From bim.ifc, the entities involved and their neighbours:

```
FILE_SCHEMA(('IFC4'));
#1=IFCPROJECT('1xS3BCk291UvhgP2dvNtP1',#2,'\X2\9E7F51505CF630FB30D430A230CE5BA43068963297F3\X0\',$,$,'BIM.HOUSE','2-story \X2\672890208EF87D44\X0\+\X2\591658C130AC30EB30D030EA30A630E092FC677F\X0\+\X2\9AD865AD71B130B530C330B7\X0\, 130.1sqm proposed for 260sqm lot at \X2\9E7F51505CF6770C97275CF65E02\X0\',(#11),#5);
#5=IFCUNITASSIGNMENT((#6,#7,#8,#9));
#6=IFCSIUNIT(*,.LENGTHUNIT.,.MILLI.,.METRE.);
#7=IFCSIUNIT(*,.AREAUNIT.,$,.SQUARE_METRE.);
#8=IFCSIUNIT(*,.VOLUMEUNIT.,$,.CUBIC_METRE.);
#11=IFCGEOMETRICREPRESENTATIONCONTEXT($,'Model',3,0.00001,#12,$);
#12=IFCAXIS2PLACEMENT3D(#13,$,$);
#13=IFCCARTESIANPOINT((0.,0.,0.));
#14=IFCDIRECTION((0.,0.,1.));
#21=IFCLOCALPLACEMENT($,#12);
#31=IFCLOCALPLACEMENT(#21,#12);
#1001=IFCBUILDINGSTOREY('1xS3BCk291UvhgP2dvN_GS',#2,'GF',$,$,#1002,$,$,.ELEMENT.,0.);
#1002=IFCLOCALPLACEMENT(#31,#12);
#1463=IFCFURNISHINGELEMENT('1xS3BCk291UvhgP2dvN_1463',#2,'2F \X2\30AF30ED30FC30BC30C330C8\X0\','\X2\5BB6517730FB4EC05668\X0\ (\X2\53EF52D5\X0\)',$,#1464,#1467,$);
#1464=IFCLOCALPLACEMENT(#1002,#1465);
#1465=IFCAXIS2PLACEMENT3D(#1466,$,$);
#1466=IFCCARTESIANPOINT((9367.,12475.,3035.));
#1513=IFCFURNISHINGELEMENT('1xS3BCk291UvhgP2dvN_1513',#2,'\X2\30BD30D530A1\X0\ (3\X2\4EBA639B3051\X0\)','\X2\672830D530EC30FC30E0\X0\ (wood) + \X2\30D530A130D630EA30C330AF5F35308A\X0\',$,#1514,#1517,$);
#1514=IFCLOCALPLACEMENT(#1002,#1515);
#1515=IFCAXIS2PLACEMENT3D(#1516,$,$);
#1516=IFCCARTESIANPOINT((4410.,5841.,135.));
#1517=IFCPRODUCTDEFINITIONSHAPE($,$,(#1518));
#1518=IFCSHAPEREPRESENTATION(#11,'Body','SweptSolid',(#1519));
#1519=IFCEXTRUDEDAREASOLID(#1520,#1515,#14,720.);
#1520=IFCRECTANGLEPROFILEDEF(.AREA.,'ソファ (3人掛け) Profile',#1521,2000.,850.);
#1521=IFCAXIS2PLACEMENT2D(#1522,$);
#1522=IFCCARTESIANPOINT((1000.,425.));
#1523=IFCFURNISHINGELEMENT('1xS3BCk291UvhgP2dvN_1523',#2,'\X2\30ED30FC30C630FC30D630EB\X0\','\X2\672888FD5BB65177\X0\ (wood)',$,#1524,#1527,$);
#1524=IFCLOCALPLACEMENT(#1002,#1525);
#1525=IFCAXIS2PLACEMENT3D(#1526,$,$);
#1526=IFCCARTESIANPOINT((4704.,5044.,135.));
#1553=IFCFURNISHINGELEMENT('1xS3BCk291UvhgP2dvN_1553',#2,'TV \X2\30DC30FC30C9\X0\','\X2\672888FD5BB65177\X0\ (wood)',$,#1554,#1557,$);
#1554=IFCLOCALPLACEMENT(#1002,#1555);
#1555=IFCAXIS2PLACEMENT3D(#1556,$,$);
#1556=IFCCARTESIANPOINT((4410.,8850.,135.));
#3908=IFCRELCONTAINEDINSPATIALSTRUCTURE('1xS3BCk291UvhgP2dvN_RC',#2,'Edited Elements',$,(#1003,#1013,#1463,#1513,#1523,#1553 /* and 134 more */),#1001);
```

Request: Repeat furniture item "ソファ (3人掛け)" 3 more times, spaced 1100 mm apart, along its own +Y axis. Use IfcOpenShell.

```python
import ifcopenshell
import ifcopenshell.api.geometry
import ifcopenshell.api.root
import ifcopenshell.util.element
import ifcopenshell.util.placement
import ifcopenshell.util.unit

model = ifcopenshell.open("bim.ifc")
unit_scale = ifcopenshell.util.unit.calculate_unit_scale(model)


def reuse_history(source, copy):
    """copy_class also copies each property set's owner history, people and application; keep the originals."""
    for rel in copy.IsDefinedBy:
        if rel.is_a("IfcRelDefinesByProperties") and (history := rel.RelatingPropertyDefinition.OwnerHistory):
            rel.RelatingPropertyDefinition.OwnerHistory = source.OwnerHistory
            ifcopenshell.util.element.remove_deep2(model, history)


source = model.by_id(1513)
base = ifcopenshell.util.placement.get_local_placement(source.ObjectPlacement)
step = base[:3, 1] * 1.1 / unit_scale

for i in range(1, 4):
    copy = ifcopenshell.api.root.copy_class(model, product=source)
    copy.Representation = ifcopenshell.util.element.copy_deep(
        model, source.Representation, exclude=["IfcGeometricRepresentationContext", "IfcRepresentationMap"]
    )
    reuse_history(source, copy)
    matrix = base.copy()
    matrix[:3, 3] += i * step
    print("added at", matrix[:3, 3].round(3) + 0.0)
    ifcopenshell.api.geometry.edit_object_placement(model, product=copy, matrix=matrix, is_si=False)

model.write("bim_rev.ifc")
```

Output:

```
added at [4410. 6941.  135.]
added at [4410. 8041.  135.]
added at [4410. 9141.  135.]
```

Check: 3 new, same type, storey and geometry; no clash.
